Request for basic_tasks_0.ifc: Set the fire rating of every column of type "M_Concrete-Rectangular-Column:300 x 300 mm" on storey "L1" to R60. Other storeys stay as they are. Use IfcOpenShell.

First a look at what the model holds.

```python
import ifcopenshell
import ifcopenshell.util.element

model = ifcopenshell.open("basic_tasks_0.ifc")
print(model.schema)
storey = next(s for s in model.by_type("IfcBuildingStorey") if s.Name == "L1")
columns = [e for e in ifcopenshell.util.element.get_decomposition(storey) if e.is_a("IfcColumn")]
seen = {}
for e in columns:
    element_type = ifcopenshell.util.element.get_type(e)
    key = (element_type.Name if element_type != e and element_type else None, ifcopenshell.util.element.get_pset(e, "Pset_ColumnCommon", "FireRating"))
    seen[key] = seen.get(key, 0) + 1
for (name, value), count in sorted(seen.items(), key=str):
    print(count, "x", name, "|", value)
```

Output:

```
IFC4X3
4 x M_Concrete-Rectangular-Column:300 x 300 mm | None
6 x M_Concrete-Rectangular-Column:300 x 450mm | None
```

```python
import ifcopenshell
import ifcopenshell.api.pset
import ifcopenshell.util.element

model = ifcopenshell.open("basic_tasks_0.ifc")

storey = next(s for s in model.by_type("IfcBuildingStorey") if s.Name == "L1")
columns = [e for e in ifcopenshell.util.element.get_decomposition(storey) if e.is_a("IfcColumn")]

count = 0
for e in columns:
    element_type = ifcopenshell.util.element.get_type(e)
    if element_type in (None, e) or element_type.Name != "M_Concrete-Rectangular-Column:300 x 300 mm":
        continue
    # add_pset returns the element's existing set when there is one.
    pset = ifcopenshell.api.pset.add_pset(model, product=e, name="Pset_ColumnCommon")
    ifcopenshell.api.pset.edit_pset(model, pset=pset, properties={"FireRating": "R60"})
    count += 1

print(count, "columns updated")

model.write("basic_tasks_0_v2.ifc")
```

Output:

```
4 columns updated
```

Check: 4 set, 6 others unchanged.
